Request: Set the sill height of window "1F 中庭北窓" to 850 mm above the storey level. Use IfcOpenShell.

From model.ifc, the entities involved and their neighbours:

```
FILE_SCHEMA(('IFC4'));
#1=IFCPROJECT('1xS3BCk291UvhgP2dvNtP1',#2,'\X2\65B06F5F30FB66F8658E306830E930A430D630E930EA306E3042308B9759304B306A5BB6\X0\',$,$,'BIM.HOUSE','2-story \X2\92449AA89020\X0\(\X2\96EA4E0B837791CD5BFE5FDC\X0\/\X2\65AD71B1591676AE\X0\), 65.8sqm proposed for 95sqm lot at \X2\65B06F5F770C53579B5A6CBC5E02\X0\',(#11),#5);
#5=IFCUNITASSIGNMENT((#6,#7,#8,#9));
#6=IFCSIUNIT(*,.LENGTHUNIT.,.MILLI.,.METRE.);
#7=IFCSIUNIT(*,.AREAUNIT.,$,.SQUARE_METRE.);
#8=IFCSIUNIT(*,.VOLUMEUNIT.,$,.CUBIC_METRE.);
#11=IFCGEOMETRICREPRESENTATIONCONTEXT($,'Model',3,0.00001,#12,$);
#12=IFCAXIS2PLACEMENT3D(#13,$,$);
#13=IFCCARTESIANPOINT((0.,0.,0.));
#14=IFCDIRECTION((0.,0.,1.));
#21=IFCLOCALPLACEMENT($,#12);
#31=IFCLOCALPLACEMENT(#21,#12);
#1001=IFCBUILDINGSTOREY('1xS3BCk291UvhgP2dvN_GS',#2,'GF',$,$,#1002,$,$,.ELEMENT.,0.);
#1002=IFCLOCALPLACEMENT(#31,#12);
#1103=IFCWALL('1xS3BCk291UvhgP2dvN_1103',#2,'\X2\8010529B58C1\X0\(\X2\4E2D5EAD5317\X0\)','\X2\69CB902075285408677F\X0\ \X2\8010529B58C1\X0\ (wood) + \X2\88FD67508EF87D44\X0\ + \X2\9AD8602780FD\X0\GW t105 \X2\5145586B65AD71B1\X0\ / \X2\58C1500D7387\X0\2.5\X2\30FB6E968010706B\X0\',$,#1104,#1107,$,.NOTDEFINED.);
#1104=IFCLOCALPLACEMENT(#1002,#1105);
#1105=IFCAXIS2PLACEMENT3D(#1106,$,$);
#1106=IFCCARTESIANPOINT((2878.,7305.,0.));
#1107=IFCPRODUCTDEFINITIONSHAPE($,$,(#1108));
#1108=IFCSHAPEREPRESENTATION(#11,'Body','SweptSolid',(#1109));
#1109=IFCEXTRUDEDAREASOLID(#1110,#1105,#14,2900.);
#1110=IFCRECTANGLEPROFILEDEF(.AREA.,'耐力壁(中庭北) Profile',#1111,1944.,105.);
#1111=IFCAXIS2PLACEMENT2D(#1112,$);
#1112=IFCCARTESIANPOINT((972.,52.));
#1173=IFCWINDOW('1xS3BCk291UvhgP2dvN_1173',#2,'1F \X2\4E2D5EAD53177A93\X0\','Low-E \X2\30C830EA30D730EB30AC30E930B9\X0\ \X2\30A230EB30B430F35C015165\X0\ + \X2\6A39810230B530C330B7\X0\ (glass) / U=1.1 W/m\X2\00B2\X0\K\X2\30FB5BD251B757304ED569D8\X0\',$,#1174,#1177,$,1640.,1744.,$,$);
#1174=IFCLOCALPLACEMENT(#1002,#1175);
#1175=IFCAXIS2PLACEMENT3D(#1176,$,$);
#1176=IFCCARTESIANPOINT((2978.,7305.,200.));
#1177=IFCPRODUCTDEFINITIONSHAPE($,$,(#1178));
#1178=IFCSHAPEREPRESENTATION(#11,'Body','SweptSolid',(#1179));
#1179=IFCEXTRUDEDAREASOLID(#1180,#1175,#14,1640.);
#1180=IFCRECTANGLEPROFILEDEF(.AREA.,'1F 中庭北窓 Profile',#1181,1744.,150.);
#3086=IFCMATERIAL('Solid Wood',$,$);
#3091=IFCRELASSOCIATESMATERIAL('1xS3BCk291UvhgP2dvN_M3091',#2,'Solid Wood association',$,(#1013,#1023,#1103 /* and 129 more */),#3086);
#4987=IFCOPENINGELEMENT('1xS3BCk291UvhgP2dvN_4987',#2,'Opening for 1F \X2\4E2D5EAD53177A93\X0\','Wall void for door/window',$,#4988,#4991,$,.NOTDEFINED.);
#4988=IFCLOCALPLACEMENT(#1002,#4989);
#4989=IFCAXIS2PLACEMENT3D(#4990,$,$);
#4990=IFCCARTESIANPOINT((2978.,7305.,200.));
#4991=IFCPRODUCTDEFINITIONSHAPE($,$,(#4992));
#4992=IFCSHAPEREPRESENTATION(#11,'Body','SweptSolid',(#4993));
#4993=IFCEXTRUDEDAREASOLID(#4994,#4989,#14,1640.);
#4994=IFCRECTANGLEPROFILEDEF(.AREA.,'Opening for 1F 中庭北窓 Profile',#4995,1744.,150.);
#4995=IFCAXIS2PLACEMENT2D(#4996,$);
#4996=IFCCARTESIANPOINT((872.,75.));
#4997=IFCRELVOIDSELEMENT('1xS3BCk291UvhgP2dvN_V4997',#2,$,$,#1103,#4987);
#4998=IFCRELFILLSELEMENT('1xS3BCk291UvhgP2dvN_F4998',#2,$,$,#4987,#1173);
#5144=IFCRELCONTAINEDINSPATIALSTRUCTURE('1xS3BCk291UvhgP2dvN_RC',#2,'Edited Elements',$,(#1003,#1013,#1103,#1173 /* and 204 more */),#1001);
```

```python
import numpy as np
import ifcopenshell
import ifcopenshell.api.geometry
import ifcopenshell.geom
import ifcopenshell.util.element
import ifcopenshell.util.placement
import ifcopenshell.util.shape
import ifcopenshell.util.unit

model = ifcopenshell.open("model.ifc")
unit_scale = ifcopenshell.util.unit.calculate_unit_scale(model)

window = model.by_guid("1xS3BCk291UvhgP2dvN_1173")
opening = window.FillsVoids[0].RelatingOpeningElement
storey = ifcopenshell.util.element.get_container(window, ifc_class="IfcBuildingStorey")
level = ifcopenshell.util.placement.get_local_placement(storey.ObjectPlacement)[2, 3]

# The opening's origin need not be at the sill, so measure its lowest point.
shape = ifcopenshell.geom.create_shape(ifcopenshell.geom.settings(), opening)
bottom = ifcopenshell.util.shape.get_shape_bottom_elevation(shape, shape.geometry) / unit_scale
dz = level + 0.85 / unit_scale - bottom

shift = np.array([0.0, 0.0, dz])
# The window is not placed relative to its opening, so move both.
for product in (opening, window):
    matrix = ifcopenshell.util.placement.get_local_placement(product.ObjectPlacement)
    matrix[:3, 3] += shift
    ifcopenshell.api.geometry.edit_object_placement(model, product=product, matrix=matrix, is_si=False)

print(f"moved by {dz * unit_scale:+.3f} m")

model.write("model_rev.ifc")
```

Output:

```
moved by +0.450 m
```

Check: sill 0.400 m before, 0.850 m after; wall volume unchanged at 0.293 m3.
